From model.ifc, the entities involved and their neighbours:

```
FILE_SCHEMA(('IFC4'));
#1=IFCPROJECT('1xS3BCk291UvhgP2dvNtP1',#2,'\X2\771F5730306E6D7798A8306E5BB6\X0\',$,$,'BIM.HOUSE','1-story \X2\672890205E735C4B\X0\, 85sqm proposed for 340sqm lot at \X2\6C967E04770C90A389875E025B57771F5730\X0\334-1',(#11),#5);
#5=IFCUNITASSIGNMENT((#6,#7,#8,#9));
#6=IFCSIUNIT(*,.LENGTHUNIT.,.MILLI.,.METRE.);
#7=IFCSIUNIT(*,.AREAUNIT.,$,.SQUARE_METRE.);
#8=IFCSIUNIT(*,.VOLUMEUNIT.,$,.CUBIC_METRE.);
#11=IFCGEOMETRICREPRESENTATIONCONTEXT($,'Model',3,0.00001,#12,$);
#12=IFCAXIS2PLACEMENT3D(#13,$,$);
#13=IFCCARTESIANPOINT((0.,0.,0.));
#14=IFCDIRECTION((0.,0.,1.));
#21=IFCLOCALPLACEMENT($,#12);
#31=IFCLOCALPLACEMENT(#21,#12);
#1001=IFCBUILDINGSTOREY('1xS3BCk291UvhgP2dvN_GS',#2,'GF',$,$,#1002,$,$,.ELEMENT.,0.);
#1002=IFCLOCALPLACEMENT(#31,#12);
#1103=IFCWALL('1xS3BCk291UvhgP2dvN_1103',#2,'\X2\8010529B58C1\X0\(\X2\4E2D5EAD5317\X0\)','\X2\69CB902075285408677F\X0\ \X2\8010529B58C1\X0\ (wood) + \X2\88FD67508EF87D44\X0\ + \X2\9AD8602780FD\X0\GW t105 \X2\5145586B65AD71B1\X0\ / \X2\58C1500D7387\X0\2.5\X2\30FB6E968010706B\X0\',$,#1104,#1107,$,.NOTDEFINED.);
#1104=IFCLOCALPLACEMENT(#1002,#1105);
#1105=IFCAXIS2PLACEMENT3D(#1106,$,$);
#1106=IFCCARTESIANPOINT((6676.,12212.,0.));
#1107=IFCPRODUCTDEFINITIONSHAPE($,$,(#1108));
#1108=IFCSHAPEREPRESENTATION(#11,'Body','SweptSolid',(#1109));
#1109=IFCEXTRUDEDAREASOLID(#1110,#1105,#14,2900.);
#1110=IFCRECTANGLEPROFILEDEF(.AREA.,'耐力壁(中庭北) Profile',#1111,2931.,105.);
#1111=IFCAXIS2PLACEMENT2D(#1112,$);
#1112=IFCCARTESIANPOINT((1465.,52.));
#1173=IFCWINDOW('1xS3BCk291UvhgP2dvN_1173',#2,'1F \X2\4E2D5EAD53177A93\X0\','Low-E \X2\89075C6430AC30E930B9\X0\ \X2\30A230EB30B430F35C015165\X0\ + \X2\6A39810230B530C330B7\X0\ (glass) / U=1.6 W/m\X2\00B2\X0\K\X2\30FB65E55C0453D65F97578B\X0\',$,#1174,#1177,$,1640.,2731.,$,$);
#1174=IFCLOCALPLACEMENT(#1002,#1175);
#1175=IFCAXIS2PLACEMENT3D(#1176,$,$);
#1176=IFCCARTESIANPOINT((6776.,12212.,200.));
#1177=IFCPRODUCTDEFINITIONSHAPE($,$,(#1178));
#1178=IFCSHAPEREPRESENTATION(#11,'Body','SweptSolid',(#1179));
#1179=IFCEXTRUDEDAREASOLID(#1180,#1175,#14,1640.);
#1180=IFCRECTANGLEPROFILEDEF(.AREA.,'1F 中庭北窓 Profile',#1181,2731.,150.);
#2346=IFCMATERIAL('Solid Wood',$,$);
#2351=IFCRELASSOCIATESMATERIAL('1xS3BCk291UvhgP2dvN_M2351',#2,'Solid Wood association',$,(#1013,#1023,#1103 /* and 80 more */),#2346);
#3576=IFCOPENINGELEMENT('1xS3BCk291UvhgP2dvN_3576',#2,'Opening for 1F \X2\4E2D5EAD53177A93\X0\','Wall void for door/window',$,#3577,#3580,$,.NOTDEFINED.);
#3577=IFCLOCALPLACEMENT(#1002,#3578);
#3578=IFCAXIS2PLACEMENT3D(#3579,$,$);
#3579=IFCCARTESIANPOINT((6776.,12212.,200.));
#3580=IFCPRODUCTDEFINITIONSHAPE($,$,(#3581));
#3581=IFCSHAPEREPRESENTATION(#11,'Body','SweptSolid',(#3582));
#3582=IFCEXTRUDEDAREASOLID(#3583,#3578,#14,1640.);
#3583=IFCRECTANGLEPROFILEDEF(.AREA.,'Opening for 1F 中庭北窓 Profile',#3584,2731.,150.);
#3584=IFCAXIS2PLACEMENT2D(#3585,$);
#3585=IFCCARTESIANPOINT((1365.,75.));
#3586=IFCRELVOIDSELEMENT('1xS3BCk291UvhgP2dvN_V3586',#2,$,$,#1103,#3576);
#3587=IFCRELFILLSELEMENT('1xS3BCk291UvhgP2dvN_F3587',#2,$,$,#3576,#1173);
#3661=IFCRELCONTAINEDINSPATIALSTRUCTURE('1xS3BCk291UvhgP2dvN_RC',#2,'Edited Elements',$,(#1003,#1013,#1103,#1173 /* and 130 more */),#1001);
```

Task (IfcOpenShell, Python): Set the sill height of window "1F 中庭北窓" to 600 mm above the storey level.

```python
import numpy as np
import ifcopenshell
import ifcopenshell.api.geometry
import ifcopenshell.geom
import ifcopenshell.util.element
import ifcopenshell.util.placement
import ifcopenshell.util.shape
import ifcopenshell.util.unit

model = ifcopenshell.open("model.ifc")
unit_scale = ifcopenshell.util.unit.calculate_unit_scale(model)

window = model.by_id(1173)
opening = window.FillsVoids[0].RelatingOpeningElement
storey = ifcopenshell.util.element.get_container(window, ifc_class="IfcBuildingStorey")
level = ifcopenshell.util.placement.get_local_placement(storey.ObjectPlacement)[2, 3]

# The opening's origin need not be at the sill, so measure its lowest point.
shape = ifcopenshell.geom.create_shape(ifcopenshell.geom.settings(), opening)
bottom = ifcopenshell.util.shape.get_shape_bottom_elevation(shape, shape.geometry) / unit_scale
dz = level + 600.0 - bottom

shift = np.array([0.0, 0.0, dz])
# The window is not placed relative to its opening, so move both.
for product in (opening, window):
    matrix = ifcopenshell.util.placement.get_local_placement(product.ObjectPlacement)
    matrix[:3, 3] += shift
    ifcopenshell.api.geometry.edit_object_placement(model, product=product, matrix=matrix, is_si=False)

print(f"moved by {dz * unit_scale:+.3f} m")

model.write("model_edited.ifc")
```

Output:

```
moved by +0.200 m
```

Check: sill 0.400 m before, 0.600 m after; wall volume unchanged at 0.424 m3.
